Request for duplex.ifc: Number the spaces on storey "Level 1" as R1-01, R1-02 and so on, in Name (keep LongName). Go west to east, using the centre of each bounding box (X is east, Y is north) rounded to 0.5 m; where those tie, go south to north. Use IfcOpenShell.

First a look at what the model holds.

```python
import ifcopenshell
import ifcopenshell.util.element
import ifcopenshell.util.placement

model = ifcopenshell.open("duplex.ifc")
print(model.schema)
storey = next(s for s in model.by_type("IfcBuildingStorey") if s.Name == "Level 1")
spaces = [e for e in ifcopenshell.util.element.get_decomposition(storey) if e.is_a("IfcSpace")]
for e in sorted(spaces, key=lambda e: e.id()):
    origin = ifcopenshell.util.placement.get_local_placement(e.ObjectPlacement)[:3, 3]
    print(e.id(), e.Name, e.LongName, origin.round(2) + 0.0, sep=" | ")
```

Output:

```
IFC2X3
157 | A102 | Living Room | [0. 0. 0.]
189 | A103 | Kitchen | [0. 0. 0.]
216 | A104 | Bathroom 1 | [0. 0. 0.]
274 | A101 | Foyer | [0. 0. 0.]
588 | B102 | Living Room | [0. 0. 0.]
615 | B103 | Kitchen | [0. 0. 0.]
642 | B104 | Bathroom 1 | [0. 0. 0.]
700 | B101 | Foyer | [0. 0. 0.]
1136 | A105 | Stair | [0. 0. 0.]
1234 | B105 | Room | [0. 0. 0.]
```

```python
import ifcopenshell
import ifcopenshell.geom
import ifcopenshell.util.element
import ifcopenshell.util.shape

model = ifcopenshell.open("duplex.ifc")
settings = ifcopenshell.geom.settings()
settings.set("use-world-coords", True)


def centre(element):
    shape = ifcopenshell.geom.create_shape(settings, element)
    return ifcopenshell.util.shape.get_bbox_centroid(shape.geometry)


storey = next(s for s in model.by_type("IfcBuildingStorey") if s.Name == "Level 1")
spaces = [e for e in ifcopenshell.util.element.get_decomposition(storey) if e.is_a("IfcSpace")]

# Insertion points can sit at a corner or the storey origin, so sort by the geometry (in metres).
centres = {e: centre(e) for e in spaces}
spaces.sort(key=lambda e: (round(centres[e][0] / 0.5), centres[e][1]))

for i, e in enumerate(spaces, start=1):
    number = f"R1-{i:02d}"
    e.Name = number
    print(e.id(), number)

model.write("duplex-out.ifc")
```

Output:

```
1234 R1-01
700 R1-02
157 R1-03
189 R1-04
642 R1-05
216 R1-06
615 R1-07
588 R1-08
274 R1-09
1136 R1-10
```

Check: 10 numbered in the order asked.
